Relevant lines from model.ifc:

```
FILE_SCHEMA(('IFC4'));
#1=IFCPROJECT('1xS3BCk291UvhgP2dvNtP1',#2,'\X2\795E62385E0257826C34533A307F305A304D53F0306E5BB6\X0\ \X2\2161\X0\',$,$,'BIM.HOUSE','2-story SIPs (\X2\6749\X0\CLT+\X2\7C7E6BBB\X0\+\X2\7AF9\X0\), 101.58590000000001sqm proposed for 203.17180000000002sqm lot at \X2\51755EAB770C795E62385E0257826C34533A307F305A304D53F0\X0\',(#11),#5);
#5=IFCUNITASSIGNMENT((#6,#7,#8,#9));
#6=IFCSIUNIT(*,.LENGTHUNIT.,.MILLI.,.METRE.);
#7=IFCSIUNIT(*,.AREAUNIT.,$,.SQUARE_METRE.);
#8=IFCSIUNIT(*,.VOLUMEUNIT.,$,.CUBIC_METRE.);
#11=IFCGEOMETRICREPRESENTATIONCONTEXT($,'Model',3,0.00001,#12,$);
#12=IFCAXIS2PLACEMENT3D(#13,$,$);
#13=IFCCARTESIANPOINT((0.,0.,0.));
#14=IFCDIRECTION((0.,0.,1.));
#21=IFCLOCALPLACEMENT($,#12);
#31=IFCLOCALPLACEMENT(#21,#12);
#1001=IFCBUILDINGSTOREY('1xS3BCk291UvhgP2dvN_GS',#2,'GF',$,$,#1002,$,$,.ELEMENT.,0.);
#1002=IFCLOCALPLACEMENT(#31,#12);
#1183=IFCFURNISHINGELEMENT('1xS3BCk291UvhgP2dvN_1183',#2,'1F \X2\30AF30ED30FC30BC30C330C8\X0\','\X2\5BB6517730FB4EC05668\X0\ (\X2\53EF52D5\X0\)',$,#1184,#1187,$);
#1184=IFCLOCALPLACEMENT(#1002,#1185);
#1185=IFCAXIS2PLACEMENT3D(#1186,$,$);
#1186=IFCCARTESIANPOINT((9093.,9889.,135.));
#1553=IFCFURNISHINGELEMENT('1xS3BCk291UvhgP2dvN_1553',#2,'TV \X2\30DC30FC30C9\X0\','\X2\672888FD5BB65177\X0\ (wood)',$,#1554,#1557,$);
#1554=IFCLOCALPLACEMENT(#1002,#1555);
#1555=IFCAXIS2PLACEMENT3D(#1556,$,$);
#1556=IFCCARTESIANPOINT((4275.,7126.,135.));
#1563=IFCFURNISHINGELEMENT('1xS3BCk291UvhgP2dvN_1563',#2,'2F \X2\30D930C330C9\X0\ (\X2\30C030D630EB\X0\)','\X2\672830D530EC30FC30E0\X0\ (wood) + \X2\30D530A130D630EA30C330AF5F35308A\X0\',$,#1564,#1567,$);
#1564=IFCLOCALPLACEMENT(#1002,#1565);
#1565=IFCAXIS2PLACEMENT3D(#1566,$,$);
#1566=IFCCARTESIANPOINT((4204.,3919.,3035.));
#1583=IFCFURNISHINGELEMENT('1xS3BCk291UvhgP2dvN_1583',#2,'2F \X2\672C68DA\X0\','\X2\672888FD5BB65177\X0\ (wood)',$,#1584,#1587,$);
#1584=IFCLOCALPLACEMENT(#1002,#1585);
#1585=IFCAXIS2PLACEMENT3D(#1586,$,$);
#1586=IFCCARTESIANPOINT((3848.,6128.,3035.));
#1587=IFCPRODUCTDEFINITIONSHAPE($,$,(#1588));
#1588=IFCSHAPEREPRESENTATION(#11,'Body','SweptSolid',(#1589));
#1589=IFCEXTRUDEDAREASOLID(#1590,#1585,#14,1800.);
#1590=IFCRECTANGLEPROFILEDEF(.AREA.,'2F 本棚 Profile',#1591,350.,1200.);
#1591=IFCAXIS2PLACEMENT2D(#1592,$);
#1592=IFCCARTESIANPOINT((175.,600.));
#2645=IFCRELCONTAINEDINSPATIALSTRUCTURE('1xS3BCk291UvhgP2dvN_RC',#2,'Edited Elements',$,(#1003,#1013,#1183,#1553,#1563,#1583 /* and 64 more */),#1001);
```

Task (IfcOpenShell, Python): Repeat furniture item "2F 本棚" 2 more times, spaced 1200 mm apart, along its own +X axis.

```python
import ifcopenshell
import ifcopenshell.api.geometry
import ifcopenshell.api.root
import ifcopenshell.util.element
import ifcopenshell.util.placement
import ifcopenshell.util.unit

model = ifcopenshell.open("model.ifc")
unit_scale = ifcopenshell.util.unit.calculate_unit_scale(model)


def reuse_history(source, copy):
    """copy_class also copies each property set's owner history, people and application; keep the originals."""
    for rel in copy.IsDefinedBy:
        if rel.is_a("IfcRelDefinesByProperties") and (history := rel.RelatingPropertyDefinition.OwnerHistory):
            rel.RelatingPropertyDefinition.OwnerHistory = source.OwnerHistory
            ifcopenshell.util.element.remove_deep2(model, history)


source = model.by_guid("1xS3BCk291UvhgP2dvN_1583")
base = ifcopenshell.util.placement.get_local_placement(source.ObjectPlacement)
step = base[:3, 0] * 1.2 / unit_scale

for i in range(1, 3):
    copy = ifcopenshell.api.root.copy_class(model, product=source)
    copy.Representation = ifcopenshell.util.element.copy_deep(
        model, source.Representation, exclude=["IfcGeometricRepresentationContext", "IfcRepresentationMap"]
    )
    reuse_history(source, copy)
    matrix = base.copy()
    matrix[:3, 3] += i * step
    print("added at", matrix[:3, 3].round(3) + 0.0)
    ifcopenshell.api.geometry.edit_object_placement(model, product=copy, matrix=matrix, is_si=False)

model.write("model-out.ifc")
```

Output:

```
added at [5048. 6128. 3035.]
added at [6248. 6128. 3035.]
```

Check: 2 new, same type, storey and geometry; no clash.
